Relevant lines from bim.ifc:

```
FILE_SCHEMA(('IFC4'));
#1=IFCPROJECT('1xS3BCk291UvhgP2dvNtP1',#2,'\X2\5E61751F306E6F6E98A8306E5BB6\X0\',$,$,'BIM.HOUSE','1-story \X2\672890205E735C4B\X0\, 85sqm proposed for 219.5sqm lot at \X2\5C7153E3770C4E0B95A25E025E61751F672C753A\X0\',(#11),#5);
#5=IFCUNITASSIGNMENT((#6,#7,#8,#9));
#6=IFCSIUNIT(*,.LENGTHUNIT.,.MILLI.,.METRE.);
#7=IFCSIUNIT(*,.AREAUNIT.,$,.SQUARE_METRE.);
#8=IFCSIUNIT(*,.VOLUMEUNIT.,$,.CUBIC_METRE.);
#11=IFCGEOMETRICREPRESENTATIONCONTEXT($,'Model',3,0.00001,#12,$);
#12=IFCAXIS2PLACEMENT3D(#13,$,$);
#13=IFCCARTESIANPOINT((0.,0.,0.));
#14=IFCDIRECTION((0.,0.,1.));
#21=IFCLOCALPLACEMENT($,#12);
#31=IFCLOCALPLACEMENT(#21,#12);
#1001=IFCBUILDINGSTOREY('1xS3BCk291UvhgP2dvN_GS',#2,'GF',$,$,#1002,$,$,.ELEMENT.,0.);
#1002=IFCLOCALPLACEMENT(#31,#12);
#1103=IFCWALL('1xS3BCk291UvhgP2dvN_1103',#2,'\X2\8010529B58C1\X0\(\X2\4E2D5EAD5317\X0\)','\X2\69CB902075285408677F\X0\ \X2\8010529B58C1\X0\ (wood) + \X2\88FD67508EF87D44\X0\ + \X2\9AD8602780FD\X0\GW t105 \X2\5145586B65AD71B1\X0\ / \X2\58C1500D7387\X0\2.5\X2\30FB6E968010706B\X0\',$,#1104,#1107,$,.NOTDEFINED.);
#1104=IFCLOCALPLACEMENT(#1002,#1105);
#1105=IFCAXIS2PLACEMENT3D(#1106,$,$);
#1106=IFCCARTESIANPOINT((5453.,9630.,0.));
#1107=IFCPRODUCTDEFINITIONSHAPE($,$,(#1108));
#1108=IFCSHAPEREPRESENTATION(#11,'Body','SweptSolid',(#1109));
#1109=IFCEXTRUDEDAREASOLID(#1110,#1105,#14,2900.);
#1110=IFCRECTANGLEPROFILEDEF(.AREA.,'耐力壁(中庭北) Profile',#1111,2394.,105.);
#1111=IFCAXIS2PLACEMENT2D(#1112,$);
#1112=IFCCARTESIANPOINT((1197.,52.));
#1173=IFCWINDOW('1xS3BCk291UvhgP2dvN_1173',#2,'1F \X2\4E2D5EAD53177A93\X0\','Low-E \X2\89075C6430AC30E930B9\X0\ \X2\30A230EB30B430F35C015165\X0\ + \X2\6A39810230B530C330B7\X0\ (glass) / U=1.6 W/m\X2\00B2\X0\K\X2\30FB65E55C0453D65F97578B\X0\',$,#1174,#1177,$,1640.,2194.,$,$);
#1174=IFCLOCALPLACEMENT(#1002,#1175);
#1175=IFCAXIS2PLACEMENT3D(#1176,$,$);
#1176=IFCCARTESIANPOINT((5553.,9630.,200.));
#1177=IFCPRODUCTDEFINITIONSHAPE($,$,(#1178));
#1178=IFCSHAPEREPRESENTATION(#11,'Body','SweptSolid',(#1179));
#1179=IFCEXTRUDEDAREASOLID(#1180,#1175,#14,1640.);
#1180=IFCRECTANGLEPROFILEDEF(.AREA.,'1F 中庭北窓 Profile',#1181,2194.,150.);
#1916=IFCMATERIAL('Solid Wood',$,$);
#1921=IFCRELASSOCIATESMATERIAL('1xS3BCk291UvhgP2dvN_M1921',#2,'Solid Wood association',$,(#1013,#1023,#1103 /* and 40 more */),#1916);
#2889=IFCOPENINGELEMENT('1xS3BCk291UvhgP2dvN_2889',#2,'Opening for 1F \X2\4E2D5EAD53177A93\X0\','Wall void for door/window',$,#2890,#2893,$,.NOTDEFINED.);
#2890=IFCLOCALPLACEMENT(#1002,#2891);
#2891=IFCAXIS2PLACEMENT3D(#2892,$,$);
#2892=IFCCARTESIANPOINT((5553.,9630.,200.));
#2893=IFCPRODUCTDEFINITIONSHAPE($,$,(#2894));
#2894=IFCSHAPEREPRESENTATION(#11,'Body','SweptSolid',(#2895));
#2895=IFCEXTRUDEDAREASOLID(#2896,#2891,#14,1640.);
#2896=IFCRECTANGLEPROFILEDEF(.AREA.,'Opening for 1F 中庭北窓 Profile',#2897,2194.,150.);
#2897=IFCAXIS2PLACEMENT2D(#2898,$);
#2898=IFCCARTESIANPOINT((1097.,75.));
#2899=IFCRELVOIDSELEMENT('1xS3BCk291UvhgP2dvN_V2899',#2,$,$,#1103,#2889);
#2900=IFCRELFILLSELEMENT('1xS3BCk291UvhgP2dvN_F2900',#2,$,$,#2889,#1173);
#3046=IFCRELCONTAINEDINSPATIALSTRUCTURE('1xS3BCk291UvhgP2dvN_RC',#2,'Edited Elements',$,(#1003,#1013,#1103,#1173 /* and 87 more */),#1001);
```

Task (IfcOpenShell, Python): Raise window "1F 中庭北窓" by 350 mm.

```python
import numpy as np
import ifcopenshell
import ifcopenshell.api.geometry
import ifcopenshell.util.placement
import ifcopenshell.util.unit

model = ifcopenshell.open("bim.ifc")
unit_scale = ifcopenshell.util.unit.calculate_unit_scale(model)

window = model.by_guid("1xS3BCk291UvhgP2dvN_1173")
opening = window.FillsVoids[0].RelatingOpeningElement
dz = 0.35 / unit_scale

shift = np.array([0.0, 0.0, dz])
# The window is not placed relative to its opening, so move both.
for product in (opening, window):
    matrix = ifcopenshell.util.placement.get_local_placement(product.ObjectPlacement)
    matrix[:3, 3] += shift
    ifcopenshell.api.geometry.edit_object_placement(model, product=product, matrix=matrix, is_si=False)

print(f"moved by {dz * unit_scale:+.3f} m")

model.write("bim_updated.ifc")
```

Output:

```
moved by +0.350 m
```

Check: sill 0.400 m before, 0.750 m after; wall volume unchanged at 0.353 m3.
